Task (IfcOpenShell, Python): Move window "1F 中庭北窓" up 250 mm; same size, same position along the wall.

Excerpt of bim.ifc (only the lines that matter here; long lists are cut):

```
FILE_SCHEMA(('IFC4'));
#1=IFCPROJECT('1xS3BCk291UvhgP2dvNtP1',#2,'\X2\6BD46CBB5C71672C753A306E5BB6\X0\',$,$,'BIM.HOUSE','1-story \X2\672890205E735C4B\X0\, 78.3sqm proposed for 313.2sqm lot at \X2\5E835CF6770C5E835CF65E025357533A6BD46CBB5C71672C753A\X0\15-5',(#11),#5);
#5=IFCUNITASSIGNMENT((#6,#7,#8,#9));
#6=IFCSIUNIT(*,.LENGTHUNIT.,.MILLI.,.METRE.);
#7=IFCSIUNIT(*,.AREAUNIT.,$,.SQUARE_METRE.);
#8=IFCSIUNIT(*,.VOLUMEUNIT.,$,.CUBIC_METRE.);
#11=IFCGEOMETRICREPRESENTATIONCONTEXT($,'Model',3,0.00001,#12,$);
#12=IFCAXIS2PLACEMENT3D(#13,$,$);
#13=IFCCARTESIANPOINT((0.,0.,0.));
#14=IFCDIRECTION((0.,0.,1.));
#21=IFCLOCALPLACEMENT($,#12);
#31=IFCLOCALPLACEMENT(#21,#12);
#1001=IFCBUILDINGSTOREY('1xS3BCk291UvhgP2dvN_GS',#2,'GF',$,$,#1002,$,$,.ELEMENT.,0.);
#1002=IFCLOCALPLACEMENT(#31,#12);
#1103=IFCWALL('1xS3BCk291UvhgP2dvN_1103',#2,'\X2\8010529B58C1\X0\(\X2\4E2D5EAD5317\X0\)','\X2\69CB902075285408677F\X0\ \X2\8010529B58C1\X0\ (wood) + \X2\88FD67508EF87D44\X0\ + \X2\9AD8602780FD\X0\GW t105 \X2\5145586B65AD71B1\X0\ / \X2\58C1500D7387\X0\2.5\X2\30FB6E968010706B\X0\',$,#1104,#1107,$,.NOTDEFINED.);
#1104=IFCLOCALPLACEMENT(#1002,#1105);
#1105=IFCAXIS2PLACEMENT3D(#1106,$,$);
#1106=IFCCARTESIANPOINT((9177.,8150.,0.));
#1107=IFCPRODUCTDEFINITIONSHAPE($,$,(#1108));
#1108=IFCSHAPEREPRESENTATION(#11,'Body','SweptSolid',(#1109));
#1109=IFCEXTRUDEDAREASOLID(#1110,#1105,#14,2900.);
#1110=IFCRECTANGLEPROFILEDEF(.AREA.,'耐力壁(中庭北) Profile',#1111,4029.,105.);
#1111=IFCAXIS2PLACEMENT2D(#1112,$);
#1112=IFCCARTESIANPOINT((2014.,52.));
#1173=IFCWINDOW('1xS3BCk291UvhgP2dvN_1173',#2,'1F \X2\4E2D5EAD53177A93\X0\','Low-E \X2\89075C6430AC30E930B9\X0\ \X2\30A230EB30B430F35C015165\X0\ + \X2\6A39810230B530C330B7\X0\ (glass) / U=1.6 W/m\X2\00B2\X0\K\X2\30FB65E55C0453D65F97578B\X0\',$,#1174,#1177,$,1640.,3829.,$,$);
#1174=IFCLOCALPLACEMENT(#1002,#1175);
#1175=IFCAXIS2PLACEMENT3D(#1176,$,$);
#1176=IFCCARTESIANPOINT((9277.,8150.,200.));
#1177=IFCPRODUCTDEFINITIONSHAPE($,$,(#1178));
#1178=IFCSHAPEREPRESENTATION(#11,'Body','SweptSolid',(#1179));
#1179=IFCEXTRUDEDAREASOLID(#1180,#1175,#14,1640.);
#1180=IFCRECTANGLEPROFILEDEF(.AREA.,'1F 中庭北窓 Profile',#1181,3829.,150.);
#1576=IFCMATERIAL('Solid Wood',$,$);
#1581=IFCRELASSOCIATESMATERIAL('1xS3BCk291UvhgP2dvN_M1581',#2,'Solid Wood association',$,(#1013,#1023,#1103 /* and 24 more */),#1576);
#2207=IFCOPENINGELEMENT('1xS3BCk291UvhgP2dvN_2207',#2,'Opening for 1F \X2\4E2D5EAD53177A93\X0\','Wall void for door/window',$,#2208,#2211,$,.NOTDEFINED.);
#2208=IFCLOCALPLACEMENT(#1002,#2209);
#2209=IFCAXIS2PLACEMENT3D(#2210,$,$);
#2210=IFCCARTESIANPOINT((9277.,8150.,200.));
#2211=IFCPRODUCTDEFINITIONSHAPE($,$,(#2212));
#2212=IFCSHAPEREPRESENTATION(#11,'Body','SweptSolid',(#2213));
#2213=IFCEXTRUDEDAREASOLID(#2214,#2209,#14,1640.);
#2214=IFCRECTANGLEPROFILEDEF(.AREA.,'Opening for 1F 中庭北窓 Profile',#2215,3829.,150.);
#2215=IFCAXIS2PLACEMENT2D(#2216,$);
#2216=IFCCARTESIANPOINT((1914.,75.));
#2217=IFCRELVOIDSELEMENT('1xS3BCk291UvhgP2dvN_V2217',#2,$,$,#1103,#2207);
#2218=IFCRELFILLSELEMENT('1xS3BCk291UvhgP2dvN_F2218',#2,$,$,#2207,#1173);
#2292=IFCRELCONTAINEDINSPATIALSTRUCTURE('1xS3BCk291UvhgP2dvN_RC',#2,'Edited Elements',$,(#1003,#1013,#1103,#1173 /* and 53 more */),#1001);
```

```python
import numpy as np
import ifcopenshell
import ifcopenshell.api.geometry
import ifcopenshell.util.placement
import ifcopenshell.util.unit

model = ifcopenshell.open("bim.ifc")
unit_scale = ifcopenshell.util.unit.calculate_unit_scale(model)

window = model.by_guid("1xS3BCk291UvhgP2dvN_1173")
opening = window.FillsVoids[0].RelatingOpeningElement
dz = 0.25 / unit_scale

shift = np.array([0.0, 0.0, dz])
# The window is not placed relative to its opening, so move both.
for product in (opening, window):
    matrix = ifcopenshell.util.placement.get_local_placement(product.ObjectPlacement)
    matrix[:3, 3] += shift
    ifcopenshell.api.geometry.edit_object_placement(model, product=product, matrix=matrix, is_si=False)

print(f"moved by {dz * unit_scale:+.3f} m")

model.write("bim_rev.ifc")
```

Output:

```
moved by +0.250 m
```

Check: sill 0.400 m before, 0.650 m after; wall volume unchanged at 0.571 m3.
